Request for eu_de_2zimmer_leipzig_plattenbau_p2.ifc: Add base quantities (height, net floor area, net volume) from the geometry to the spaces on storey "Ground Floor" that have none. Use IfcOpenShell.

First a look at what the model holds.

```python
import ifcopenshell
import ifcopenshell.util.element
import ifcopenshell.util.unit

model = ifcopenshell.open("eu_de_2zimmer_leipzig_plattenbau_p2.ifc")
print(model.schema)
for unit_type in ("LENGTHUNIT", "AREAUNIT", "VOLUMEUNIT"):
    print(unit_type, ifcopenshell.util.unit.calculate_unit_scale(model, unit_type))
storey = next(s for s in model.by_type("IfcBuildingStorey") if s.Name == "Ground Floor")
spaces = [e for e in ifcopenshell.util.element.get_decomposition(storey) if e.is_a("IfcSpace")]
for e in sorted(spaces, key=lambda e: e.id()):
    print(e.id(), e.is_a(), e.Name, list(ifcopenshell.util.element.get_psets(e, qtos_only=True)), sep=" | ")
```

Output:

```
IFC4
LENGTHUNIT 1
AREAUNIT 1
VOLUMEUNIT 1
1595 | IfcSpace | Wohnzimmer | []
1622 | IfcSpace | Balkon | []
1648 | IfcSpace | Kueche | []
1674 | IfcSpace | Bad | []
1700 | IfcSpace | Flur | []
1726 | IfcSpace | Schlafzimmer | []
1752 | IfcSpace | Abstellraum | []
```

```python
import ifcopenshell
import ifcopenshell.api.pset
import ifcopenshell.geom
import ifcopenshell.util.element
import ifcopenshell.util.shape
import ifcopenshell.util.unit

model = ifcopenshell.open("eu_de_2zimmer_leipzig_plattenbau_p2.ifc")
unit_scale = ifcopenshell.util.unit.calculate_unit_scale(model)
area_scale = ifcopenshell.util.unit.calculate_unit_scale(model, "AREAUNIT")
volume_scale = ifcopenshell.util.unit.calculate_unit_scale(model, "VOLUMEUNIT")
settings = ifcopenshell.geom.settings()

storey = next(s for s in model.by_type("IfcBuildingStorey") if s.Name == "Ground Floor")
spaces = [e for e in ifcopenshell.util.element.get_decomposition(storey) if e.is_a("IfcSpace")]

for e in sorted(spaces, key=lambda e: e.id()):
    if ifcopenshell.util.element.get_psets(e, qtos_only=True, should_inherit=False):
        continue
    # Geometry comes back in metres, in the element's own axes.
    shape = ifcopenshell.geom.create_shape(settings, e)
    values = {
        "Height": ifcopenshell.util.shape.get_z(shape.geometry) / unit_scale,
        "NetFloorArea": ifcopenshell.util.shape.get_footprint_area(shape.geometry) / area_scale,
        "NetVolume": ifcopenshell.util.shape.get_volume(shape.geometry) / volume_scale,
    }
    qto = ifcopenshell.api.pset.add_qto(model, product=e, name="Qto_SpaceBaseQuantities")
    ifcopenshell.api.pset.edit_qto(model, qto=qto, properties=values)
    print(e.id(), {k: round(v, 3) for k, v in values.items()})

model.write("eu_de_2zimmer_leipzig_plattenbau_p2-out.ifc")
```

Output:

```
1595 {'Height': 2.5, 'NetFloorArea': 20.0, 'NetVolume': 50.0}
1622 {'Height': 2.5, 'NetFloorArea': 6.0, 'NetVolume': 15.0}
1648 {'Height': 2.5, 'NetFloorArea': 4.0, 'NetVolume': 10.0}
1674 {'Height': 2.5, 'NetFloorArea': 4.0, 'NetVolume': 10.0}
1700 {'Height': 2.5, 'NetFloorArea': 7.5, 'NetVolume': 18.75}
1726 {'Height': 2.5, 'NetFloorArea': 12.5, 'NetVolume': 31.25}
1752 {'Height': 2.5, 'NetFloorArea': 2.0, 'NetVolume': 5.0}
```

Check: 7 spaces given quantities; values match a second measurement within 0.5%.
